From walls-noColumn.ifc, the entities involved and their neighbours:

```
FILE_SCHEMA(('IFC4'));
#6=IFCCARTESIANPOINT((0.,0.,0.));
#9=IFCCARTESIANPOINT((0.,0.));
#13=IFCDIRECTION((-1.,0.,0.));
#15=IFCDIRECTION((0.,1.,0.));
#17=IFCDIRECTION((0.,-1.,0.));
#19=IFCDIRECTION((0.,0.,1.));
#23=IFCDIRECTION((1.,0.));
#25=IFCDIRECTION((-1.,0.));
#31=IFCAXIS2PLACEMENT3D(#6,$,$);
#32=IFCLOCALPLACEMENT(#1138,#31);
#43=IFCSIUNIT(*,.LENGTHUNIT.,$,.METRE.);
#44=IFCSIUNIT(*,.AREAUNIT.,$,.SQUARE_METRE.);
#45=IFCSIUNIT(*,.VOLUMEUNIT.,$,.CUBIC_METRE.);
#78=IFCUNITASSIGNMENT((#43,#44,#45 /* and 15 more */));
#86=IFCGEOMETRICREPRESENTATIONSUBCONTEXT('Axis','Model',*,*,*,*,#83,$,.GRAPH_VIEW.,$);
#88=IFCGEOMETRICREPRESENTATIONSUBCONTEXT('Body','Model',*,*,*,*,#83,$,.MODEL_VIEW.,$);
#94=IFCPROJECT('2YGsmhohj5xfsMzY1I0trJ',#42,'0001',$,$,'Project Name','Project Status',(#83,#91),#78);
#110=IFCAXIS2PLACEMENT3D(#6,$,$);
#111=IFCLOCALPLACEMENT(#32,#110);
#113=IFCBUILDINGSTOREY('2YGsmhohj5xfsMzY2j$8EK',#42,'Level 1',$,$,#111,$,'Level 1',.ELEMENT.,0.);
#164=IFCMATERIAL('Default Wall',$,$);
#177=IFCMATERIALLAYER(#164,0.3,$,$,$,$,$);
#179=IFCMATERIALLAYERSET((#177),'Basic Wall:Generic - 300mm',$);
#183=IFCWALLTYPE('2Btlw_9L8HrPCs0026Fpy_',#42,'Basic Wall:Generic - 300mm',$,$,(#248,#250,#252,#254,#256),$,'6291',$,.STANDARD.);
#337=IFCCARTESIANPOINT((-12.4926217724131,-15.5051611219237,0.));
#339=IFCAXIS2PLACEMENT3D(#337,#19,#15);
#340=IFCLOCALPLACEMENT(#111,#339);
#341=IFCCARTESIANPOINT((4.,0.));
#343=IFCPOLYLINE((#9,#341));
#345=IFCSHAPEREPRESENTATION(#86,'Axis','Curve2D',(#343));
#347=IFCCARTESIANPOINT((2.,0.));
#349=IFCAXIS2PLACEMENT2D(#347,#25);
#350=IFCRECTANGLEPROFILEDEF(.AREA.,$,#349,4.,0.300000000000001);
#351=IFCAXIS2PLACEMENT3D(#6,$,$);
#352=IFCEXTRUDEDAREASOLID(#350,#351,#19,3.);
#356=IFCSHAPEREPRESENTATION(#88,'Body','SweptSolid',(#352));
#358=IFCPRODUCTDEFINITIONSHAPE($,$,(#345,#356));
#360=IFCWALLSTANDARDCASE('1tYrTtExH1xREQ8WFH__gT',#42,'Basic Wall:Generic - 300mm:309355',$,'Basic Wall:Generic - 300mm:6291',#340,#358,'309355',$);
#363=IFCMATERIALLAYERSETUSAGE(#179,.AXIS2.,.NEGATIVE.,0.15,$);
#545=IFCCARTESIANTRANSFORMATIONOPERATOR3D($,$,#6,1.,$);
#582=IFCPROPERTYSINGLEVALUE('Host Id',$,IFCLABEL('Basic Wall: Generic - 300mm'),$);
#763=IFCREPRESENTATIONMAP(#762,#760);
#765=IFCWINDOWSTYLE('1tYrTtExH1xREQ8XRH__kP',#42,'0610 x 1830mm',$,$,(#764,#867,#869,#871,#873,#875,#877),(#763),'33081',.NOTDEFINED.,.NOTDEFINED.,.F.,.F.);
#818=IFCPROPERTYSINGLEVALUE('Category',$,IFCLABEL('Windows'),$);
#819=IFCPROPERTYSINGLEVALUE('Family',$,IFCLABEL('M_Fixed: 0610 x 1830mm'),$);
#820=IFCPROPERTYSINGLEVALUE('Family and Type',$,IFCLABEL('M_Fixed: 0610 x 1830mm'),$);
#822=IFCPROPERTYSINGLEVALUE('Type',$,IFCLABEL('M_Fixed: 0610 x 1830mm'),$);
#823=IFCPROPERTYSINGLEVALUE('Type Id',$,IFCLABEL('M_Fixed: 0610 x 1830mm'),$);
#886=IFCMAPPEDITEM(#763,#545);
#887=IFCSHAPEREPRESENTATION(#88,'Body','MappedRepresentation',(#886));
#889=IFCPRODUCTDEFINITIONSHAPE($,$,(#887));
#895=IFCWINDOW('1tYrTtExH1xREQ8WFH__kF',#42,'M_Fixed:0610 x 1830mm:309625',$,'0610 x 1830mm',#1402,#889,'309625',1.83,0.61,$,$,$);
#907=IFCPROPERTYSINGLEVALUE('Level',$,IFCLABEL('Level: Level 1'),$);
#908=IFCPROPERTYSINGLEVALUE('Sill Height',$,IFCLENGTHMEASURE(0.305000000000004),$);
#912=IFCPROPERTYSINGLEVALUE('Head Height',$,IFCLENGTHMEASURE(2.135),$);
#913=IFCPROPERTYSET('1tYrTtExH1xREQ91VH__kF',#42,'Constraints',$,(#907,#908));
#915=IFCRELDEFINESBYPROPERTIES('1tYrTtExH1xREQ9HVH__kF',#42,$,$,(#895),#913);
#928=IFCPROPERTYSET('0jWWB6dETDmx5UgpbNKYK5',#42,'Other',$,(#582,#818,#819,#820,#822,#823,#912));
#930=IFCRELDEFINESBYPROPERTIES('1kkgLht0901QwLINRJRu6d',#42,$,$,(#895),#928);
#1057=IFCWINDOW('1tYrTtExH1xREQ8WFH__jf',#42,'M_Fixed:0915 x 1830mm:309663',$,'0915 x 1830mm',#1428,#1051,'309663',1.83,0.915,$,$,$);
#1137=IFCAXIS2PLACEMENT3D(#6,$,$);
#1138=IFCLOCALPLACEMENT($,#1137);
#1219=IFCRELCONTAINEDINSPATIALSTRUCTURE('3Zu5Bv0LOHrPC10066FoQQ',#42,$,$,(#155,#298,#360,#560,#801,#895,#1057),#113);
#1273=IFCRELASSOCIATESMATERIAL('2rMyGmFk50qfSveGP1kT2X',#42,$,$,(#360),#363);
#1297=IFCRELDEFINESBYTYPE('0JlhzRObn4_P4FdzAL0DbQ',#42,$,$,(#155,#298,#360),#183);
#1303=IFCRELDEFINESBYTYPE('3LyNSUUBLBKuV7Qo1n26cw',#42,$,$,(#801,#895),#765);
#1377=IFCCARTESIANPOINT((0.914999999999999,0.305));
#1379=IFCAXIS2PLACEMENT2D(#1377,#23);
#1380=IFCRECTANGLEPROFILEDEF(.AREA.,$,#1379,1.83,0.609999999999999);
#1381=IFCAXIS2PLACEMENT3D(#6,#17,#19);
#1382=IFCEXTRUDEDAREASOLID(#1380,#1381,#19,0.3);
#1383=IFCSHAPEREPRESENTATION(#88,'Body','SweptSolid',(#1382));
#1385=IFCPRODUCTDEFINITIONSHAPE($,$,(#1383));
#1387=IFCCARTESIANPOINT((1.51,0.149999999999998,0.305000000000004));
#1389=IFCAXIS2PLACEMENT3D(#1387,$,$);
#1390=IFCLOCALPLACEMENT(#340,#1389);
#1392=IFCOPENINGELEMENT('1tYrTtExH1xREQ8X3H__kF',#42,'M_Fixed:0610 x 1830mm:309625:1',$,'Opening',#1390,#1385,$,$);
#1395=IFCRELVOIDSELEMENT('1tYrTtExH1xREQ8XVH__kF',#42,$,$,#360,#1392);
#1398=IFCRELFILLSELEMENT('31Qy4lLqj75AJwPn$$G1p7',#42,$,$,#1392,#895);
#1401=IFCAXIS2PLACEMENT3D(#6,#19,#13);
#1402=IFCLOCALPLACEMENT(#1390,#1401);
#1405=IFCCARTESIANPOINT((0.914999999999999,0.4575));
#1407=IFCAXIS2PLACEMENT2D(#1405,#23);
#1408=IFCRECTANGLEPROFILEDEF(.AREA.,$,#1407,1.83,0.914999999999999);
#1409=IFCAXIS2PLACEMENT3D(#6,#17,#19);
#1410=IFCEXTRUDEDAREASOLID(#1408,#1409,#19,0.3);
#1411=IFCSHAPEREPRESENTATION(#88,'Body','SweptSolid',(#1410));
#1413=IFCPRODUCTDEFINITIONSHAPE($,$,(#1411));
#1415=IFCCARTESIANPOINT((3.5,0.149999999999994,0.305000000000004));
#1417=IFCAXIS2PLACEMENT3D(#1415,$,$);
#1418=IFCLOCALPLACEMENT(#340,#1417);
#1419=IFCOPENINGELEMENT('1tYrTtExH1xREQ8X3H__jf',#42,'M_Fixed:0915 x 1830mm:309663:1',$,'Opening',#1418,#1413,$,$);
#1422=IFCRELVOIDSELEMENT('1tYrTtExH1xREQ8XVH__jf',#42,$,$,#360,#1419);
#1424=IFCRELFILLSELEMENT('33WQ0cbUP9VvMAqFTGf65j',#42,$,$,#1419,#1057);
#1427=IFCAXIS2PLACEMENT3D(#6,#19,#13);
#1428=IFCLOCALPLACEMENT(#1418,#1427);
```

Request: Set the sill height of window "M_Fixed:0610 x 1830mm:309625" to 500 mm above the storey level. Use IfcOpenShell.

```python
import numpy as np
import ifcopenshell
import ifcopenshell.api.geometry
import ifcopenshell.api.pset
import ifcopenshell.geom
import ifcopenshell.util.element
import ifcopenshell.util.placement
import ifcopenshell.util.shape
import ifcopenshell.util.unit

model = ifcopenshell.open("walls-noColumn.ifc")
unit_scale = ifcopenshell.util.unit.calculate_unit_scale(model)

window = model.by_id(895)
opening = window.FillsVoids[0].RelatingOpeningElement
storey = ifcopenshell.util.element.get_container(window, ifc_class="IfcBuildingStorey")
level = ifcopenshell.util.placement.get_local_placement(storey.ObjectPlacement)[2, 3]

# The opening's origin need not be at the sill, so measure its lowest point.
shape = ifcopenshell.geom.create_shape(ifcopenshell.geom.settings(), opening)
bottom = ifcopenshell.util.shape.get_shape_bottom_elevation(shape, shape.geometry) / unit_scale
dz = level + 0.5 - bottom

shift = np.array([0.0, 0.0, dz])
# The window is placed relative to its opening, so it follows when the opening moves.
matrix = ifcopenshell.util.placement.get_local_placement(opening.ObjectPlacement)
matrix[:3, 3] += shift
ifcopenshell.api.geometry.edit_object_placement(
    model, product=opening, matrix=matrix, is_si=False, should_transform_children=True
)

# Keep the stored heights in step.
pset = model.by_id(ifcopenshell.util.element.get_pset(window, "Constraints", should_inherit=False)["id"])
ifcopenshell.api.pset.edit_pset(model, pset=pset, properties={
    "Sill Height": model.create_entity("IfcLengthMeasure", ifcopenshell.util.element.get_pset(window, "Constraints", "Sill Height") + dz),
})
pset = model.by_id(ifcopenshell.util.element.get_pset(window, "Other", should_inherit=False)["id"])
ifcopenshell.api.pset.edit_pset(model, pset=pset, properties={
    "Head Height": model.create_entity("IfcLengthMeasure", ifcopenshell.util.element.get_pset(window, "Other", "Head Height") + dz),
})

print(f"moved by {dz * unit_scale:+.3f} m")

model.write("walls-noColumn_v2.ifc")
```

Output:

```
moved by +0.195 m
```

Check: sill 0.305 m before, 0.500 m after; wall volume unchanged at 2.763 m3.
